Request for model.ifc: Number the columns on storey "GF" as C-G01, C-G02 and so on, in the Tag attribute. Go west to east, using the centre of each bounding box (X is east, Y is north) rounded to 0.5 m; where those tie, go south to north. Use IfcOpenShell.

First a look at what the model holds.

```python
import ifcopenshell
import ifcopenshell.util.element
import ifcopenshell.util.placement

model = ifcopenshell.open("model.ifc")
print(model.schema)
storey = next(s for s in model.by_type("IfcBuildingStorey") if s.Name == "GF")
columns = [e for e in ifcopenshell.util.element.get_decomposition(storey) if e.is_a("IfcColumn")]
for e in sorted(columns, key=lambda e: e.id()):
    origin = ifcopenshell.util.placement.get_local_placement(e.ObjectPlacement)[:3, 3]
    print(e.id(), e.Tag, e.Name, origin.round(2) + 0.0, sep=" | ")
```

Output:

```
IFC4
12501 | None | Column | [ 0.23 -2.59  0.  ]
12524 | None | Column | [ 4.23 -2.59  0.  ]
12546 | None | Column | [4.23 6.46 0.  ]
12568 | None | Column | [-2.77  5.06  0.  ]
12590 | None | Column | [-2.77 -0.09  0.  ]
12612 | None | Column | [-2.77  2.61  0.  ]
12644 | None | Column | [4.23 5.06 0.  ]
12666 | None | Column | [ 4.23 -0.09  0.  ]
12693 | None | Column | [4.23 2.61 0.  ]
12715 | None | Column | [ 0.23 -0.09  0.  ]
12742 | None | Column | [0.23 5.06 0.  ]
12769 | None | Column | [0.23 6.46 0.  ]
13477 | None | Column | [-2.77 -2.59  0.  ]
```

```python
import ifcopenshell
import ifcopenshell.geom
import ifcopenshell.util.element
import ifcopenshell.util.shape

model = ifcopenshell.open("model.ifc")
settings = ifcopenshell.geom.settings()
settings.set("use-world-coords", True)


def centre(element):
    shape = ifcopenshell.geom.create_shape(settings, element)
    return ifcopenshell.util.shape.get_bbox_centroid(shape.geometry)


storey = next(s for s in model.by_type("IfcBuildingStorey") if s.Name == "GF")
columns = [e for e in ifcopenshell.util.element.get_decomposition(storey) if e.is_a("IfcColumn")]

# Insertion points can sit at a corner or the storey origin, so sort by the geometry (in metres).
centres = {e: centre(e) for e in columns}
columns.sort(key=lambda e: (round(centres[e][0] / 0.5), centres[e][1]))

for i, e in enumerate(columns, start=1):
    number = f"C-G{i:02d}"
    e.Tag = number
    print(e.id(), number)

model.write("model_updated.ifc")
```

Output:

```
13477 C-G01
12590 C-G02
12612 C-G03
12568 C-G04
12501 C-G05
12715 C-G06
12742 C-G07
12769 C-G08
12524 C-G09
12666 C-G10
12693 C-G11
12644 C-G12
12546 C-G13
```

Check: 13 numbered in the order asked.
